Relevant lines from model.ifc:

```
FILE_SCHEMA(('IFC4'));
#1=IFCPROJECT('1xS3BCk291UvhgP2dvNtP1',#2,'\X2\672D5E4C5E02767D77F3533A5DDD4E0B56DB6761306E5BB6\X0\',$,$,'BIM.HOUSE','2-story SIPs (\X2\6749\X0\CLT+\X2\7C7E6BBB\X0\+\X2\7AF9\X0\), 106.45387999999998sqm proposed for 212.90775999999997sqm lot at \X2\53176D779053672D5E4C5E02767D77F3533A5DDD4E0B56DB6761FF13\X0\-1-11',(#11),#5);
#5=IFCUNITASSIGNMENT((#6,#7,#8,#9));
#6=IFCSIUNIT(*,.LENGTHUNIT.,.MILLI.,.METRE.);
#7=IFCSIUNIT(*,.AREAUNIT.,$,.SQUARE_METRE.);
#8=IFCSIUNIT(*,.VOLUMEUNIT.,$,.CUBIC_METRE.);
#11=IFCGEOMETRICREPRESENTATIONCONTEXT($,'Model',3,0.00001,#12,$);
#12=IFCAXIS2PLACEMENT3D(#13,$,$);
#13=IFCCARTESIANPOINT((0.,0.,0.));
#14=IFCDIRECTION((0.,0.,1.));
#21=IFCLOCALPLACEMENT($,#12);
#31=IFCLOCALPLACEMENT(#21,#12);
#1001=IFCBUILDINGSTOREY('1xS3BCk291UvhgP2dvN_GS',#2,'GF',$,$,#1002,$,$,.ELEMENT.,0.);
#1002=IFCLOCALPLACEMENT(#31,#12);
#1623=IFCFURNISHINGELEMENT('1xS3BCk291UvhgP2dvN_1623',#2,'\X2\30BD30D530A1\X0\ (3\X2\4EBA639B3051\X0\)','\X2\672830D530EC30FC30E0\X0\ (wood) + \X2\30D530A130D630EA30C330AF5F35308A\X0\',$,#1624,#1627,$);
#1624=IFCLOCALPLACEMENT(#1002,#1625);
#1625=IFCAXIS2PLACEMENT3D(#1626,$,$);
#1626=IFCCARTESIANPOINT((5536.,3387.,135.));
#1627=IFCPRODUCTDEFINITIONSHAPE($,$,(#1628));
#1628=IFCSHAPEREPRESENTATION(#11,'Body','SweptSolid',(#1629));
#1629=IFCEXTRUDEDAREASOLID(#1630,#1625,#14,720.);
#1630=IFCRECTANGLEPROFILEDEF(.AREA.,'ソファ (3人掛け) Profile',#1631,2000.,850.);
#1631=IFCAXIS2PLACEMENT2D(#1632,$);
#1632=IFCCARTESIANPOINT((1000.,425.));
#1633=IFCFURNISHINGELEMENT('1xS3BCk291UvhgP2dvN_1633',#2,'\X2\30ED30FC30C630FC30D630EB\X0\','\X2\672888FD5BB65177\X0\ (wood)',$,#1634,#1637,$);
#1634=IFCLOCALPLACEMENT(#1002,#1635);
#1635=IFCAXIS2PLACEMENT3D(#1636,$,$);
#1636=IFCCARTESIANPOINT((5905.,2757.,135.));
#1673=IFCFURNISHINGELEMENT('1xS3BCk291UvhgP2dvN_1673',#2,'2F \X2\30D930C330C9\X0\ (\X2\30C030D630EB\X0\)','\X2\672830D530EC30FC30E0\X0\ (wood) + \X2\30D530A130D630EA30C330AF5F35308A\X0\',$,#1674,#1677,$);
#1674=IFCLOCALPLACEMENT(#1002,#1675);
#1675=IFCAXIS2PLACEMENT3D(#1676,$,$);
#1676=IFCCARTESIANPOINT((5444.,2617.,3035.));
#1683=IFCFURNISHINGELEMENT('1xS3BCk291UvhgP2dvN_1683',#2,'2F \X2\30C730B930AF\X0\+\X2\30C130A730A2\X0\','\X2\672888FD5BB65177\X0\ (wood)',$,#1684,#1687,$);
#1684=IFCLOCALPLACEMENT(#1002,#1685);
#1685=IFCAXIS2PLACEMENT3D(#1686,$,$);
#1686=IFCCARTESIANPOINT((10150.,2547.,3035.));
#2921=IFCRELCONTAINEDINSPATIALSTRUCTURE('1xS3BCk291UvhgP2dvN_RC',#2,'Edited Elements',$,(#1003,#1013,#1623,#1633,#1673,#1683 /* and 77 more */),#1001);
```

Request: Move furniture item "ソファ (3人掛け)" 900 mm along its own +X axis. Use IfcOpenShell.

```python
import ifcopenshell
import ifcopenshell.api.geometry
import ifcopenshell.util.placement

model = ifcopenshell.open("model.ifc")

item = model.by_id(1623)
matrix = ifcopenshell.util.placement.get_local_placement(item.ObjectPlacement)
matrix[:3, 3] += matrix[:3, 0] * 900.0
ifcopenshell.api.geometry.edit_object_placement(model, product=item, matrix=matrix, is_si=False)

print(ifcopenshell.util.placement.get_local_placement(item.ObjectPlacement).round(3) + 0.0)

model.write("model_v2.ifc")
```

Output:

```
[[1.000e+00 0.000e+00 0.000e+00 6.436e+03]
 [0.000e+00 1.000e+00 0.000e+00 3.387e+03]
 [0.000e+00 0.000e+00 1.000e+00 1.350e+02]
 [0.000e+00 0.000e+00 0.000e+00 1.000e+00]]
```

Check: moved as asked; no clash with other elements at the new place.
